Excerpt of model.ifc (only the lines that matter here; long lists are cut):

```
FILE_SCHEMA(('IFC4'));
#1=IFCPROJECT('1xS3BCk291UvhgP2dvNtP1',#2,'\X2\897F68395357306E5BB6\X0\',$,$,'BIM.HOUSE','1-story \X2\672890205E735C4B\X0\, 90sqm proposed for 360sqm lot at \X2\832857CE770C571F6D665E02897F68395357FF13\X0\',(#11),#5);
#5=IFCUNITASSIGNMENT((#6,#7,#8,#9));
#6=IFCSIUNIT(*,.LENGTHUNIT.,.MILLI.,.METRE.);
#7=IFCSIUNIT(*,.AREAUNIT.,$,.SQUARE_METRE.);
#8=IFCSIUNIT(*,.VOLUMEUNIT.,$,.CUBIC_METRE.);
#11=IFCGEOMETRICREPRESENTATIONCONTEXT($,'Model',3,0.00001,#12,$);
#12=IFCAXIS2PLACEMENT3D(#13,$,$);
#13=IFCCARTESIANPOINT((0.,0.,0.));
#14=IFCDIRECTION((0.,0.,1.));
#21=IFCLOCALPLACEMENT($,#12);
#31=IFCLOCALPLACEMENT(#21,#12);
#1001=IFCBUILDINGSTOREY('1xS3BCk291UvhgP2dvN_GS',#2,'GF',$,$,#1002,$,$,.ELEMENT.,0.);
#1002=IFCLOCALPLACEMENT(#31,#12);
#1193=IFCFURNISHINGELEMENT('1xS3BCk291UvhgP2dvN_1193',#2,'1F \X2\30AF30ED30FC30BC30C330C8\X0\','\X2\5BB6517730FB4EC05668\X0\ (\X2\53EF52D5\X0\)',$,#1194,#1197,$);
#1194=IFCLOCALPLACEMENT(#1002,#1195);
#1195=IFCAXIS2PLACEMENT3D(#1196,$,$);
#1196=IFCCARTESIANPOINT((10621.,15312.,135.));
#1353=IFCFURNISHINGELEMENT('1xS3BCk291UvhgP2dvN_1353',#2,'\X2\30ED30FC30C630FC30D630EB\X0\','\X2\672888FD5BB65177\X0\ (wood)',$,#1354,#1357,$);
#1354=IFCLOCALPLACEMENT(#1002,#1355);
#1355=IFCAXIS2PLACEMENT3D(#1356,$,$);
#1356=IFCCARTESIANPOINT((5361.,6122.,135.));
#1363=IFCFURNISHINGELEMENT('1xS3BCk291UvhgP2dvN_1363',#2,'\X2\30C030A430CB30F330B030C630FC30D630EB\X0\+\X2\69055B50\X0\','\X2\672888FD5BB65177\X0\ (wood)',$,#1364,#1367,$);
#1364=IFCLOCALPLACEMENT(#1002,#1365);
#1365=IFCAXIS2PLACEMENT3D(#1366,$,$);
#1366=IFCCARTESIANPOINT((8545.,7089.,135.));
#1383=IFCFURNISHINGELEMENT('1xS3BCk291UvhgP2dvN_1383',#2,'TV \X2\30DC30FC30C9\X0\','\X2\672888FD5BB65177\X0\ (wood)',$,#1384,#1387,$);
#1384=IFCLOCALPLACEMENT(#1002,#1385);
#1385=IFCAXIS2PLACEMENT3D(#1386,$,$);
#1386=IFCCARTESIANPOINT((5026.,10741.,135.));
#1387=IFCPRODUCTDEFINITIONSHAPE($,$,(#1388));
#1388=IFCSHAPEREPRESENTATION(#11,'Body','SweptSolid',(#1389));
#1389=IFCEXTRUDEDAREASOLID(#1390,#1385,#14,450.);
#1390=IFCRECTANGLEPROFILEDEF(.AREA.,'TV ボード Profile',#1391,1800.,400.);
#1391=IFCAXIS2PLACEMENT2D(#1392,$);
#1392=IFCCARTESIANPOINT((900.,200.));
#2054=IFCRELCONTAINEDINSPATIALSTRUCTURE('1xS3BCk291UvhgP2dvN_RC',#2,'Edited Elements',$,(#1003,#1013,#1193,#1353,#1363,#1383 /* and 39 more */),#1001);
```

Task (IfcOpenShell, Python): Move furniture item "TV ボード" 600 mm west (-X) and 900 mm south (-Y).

```python
import ifcopenshell
import ifcopenshell.api.geometry
import ifcopenshell.util.placement
import ifcopenshell.util.unit

model = ifcopenshell.open("model.ifc")
unit_scale = ifcopenshell.util.unit.calculate_unit_scale(model)

item = model.by_guid("1xS3BCk291UvhgP2dvN_1383")
matrix = ifcopenshell.util.placement.get_local_placement(item.ObjectPlacement)
matrix[0, 3] -= 0.6 / unit_scale
matrix[1, 3] -= 0.9 / unit_scale
ifcopenshell.api.geometry.edit_object_placement(model, product=item, matrix=matrix, is_si=False)

print(ifcopenshell.util.placement.get_local_placement(item.ObjectPlacement).round(3) + 0.0)

model.write("model_edited.ifc")
```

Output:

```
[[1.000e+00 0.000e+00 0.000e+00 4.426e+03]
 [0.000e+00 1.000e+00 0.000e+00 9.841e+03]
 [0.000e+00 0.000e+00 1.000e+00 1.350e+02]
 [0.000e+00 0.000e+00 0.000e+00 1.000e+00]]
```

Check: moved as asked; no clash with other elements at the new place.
